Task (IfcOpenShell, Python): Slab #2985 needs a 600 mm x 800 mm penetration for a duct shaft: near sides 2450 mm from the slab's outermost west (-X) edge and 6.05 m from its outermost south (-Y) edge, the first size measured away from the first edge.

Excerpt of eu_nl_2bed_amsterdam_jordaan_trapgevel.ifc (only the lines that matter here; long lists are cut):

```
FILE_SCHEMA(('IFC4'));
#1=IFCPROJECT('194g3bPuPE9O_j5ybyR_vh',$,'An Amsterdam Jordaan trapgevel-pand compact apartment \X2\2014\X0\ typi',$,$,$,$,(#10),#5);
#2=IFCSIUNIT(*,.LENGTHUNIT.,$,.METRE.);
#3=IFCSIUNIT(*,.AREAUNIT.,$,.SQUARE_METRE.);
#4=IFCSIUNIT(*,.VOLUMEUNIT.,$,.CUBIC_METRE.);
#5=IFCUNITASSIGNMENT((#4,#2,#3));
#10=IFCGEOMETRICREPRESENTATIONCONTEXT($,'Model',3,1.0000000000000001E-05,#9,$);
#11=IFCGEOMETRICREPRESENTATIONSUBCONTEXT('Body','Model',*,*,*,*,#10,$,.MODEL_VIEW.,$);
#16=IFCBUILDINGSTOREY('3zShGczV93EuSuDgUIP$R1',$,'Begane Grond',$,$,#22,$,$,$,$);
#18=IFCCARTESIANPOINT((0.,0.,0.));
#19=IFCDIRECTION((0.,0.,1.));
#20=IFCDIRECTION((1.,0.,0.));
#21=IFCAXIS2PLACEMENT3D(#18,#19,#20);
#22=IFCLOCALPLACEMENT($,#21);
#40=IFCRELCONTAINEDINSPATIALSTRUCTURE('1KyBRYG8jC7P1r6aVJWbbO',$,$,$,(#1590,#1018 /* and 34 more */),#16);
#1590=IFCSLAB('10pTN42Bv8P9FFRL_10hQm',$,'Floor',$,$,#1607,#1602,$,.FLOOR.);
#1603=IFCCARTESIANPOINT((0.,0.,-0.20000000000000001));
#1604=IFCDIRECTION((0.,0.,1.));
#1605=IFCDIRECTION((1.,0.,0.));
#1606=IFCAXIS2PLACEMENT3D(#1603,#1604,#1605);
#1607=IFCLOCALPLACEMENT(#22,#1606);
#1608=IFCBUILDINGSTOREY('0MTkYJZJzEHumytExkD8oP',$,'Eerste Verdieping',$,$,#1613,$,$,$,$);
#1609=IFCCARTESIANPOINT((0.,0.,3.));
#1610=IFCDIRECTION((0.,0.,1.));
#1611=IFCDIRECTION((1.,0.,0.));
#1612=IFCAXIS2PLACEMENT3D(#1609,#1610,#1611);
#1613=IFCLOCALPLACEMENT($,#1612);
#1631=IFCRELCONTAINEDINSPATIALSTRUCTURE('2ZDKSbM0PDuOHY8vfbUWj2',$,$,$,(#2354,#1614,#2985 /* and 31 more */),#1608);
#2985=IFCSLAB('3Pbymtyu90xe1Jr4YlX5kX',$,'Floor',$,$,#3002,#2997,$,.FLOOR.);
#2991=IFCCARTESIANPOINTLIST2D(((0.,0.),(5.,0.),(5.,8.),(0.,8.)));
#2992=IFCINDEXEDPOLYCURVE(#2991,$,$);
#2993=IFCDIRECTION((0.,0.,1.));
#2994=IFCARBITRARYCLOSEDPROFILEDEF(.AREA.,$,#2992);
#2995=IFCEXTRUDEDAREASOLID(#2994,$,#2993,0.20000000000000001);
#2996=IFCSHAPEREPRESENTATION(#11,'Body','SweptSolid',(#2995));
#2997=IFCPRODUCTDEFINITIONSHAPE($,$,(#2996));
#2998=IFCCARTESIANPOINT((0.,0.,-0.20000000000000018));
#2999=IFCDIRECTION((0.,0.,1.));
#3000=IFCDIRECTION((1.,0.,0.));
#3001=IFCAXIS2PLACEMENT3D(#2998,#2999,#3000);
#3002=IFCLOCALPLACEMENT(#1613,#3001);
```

```python
import numpy as np
import ifcopenshell
import ifcopenshell.api.feature
import ifcopenshell.api.geometry
import ifcopenshell.api.root
import ifcopenshell.geom
import ifcopenshell.util.placement
import ifcopenshell.util.representation
import ifcopenshell.util.shape
import ifcopenshell.util.unit

model = ifcopenshell.open("eu_nl_2bed_amsterdam_jordaan_trapgevel.ifc")
unit_scale = ifcopenshell.util.unit.calculate_unit_scale(model)
settings = ifcopenshell.geom.settings()


def volume(element):
    """Net volume in cubic metres, openings subtracted."""
    shape = ifcopenshell.geom.create_shape(settings, element)
    return ifcopenshell.util.shape.get_volume(shape.geometry)


slab = model.by_guid("3Pbymtyu90xe1Jr4YlX5kX")
before = volume(slab)

# Extent in the slab's own axes, in metres. The edges named are its -X and -Y sides.
slab_shape = ifcopenshell.geom.create_shape(settings, slab)
vertices = ifcopenshell.util.shape.get_vertices(slab_shape.geometry)
x_min, y_min, bottom = vertices.min(axis=0)
top = vertices[:, 2].max()

opening = ifcopenshell.api.root.create_entity(model, ifc_class="IfcOpeningElement", name="Duct shaft opening", predefined_type="OPENING")
context = ifcopenshell.util.representation.get_context(model, "Model", "Body", "MODEL_VIEW")
width, depth = 0.6, 0.8
outline = [(0.0, 0.0), (width, 0.0), (width, depth), (0.0, depth), (0.0, 0.0)]
# Overshoot both faces by 50 mm so the cut is clean.
shape = ifcopenshell.api.geometry.add_slab_representation(
    model, context=context, depth=top - bottom + 0.1, polyline=outline
)
ifcopenshell.api.geometry.assign_representation(model, product=opening, representation=shape)

matrix = ifcopenshell.util.placement.get_local_placement(slab.ObjectPlacement)
matrix[:, 3] = matrix @ np.append(np.array([x_min + 2.45, y_min + 6.05, bottom - 0.05]) / unit_scale, 1.0)
ifcopenshell.api.geometry.edit_object_placement(model, product=opening, matrix=matrix, is_si=False)
ifcopenshell.api.feature.add_feature(model, feature=opening, element=slab)

after = volume(slab)

print(f"slab volume {before:.3f} -> {after:.3f} m3")

model.write("eu_nl_2bed_amsterdam_jordaan_trapgevel-out.ifc")
```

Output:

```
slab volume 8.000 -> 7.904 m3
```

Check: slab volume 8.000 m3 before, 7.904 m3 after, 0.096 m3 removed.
